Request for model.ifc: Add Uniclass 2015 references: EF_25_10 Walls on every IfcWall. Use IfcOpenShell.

First a look at what the model holds.

```python
import ifcopenshell

model = ifcopenshell.open("model.ifc")
print(model.schema)
print("classifications:", [c.Name for c in model.by_type("IfcClassification")])
for ifc_class in ("IfcDoor", "IfcRoof", "IfcStair", "IfcWall", "IfcWindow"):
    print(ifc_class, len(model.by_type(ifc_class)))
```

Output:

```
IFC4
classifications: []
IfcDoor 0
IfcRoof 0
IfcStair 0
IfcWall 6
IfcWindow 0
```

```python
import ifcopenshell
import ifcopenshell.api.classification

model = ifcopenshell.open("model.ifc")

system = ifcopenshell.api.classification.add_classification(model, classification="Uniclass 2015")

codes = {
    "IfcWall": ("EF_25_10", "Walls"),
}
for ifc_class, (code, name) in codes.items():
    products = model.by_type(ifc_class)
    ifcopenshell.api.classification.add_reference(
        model, products=products, classification=system, identification=code, name=name
    )
    print(code, len(products))

model.write("model_v2.ifc")
```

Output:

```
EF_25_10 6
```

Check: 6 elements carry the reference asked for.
